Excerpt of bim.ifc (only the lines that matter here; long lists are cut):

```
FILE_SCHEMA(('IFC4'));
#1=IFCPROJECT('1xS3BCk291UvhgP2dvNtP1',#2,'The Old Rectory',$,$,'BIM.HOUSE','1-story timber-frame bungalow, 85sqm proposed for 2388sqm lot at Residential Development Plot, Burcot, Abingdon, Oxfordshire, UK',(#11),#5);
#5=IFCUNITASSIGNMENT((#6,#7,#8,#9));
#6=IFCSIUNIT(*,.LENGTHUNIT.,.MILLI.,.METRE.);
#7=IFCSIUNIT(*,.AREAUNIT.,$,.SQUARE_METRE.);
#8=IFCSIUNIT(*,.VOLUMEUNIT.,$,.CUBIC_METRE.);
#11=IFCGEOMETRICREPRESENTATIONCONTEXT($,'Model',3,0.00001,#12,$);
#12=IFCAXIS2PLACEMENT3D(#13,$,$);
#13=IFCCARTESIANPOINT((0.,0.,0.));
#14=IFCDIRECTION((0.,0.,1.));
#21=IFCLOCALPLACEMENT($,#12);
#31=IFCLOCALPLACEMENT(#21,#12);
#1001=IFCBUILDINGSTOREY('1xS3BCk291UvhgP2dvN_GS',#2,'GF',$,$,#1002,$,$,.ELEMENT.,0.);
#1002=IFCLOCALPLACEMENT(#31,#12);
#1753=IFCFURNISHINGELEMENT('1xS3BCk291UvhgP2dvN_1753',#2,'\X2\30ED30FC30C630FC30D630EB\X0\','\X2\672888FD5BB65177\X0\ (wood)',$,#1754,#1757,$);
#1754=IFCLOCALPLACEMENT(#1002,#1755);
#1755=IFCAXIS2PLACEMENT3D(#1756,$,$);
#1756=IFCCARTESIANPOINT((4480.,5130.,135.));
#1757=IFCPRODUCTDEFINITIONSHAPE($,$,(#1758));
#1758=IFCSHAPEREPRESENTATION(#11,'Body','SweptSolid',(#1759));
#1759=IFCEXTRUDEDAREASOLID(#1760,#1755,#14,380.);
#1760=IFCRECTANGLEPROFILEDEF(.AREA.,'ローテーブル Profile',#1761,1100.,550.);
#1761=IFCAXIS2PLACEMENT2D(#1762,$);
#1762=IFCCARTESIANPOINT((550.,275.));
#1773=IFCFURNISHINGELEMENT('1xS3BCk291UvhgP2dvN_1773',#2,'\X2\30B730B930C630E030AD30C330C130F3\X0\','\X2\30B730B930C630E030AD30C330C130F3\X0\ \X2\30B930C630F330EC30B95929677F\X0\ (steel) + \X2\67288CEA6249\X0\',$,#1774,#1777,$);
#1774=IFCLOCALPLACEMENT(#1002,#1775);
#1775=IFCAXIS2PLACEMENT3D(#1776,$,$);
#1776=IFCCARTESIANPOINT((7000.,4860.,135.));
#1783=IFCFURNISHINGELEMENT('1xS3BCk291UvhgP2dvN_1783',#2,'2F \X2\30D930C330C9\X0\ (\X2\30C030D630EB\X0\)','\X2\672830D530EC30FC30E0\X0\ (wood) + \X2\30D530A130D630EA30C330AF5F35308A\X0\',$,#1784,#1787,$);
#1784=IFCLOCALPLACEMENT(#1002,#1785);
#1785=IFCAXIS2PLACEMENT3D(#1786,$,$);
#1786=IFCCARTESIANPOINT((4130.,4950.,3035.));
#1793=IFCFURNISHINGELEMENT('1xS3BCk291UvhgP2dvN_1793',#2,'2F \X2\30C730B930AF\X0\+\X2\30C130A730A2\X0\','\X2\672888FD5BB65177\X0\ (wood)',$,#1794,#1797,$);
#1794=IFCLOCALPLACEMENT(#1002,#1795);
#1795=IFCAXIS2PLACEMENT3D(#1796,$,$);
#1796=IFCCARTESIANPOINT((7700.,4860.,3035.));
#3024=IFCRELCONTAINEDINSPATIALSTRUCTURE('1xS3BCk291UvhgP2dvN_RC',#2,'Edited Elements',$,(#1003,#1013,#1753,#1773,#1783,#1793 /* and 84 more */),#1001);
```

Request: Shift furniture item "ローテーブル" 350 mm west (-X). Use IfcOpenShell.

```python
import ifcopenshell
import ifcopenshell.api.geometry
import ifcopenshell.util.placement
import ifcopenshell.util.unit

model = ifcopenshell.open("bim.ifc")
unit_scale = ifcopenshell.util.unit.calculate_unit_scale(model)

item = model.by_guid("1xS3BCk291UvhgP2dvN_1753")
matrix = ifcopenshell.util.placement.get_local_placement(item.ObjectPlacement)
matrix[0, 3] -= 0.35 / unit_scale
ifcopenshell.api.geometry.edit_object_placement(model, product=item, matrix=matrix, is_si=False)

print(ifcopenshell.util.placement.get_local_placement(item.ObjectPlacement).round(3) + 0.0)

model.write("bim_edited.ifc")
```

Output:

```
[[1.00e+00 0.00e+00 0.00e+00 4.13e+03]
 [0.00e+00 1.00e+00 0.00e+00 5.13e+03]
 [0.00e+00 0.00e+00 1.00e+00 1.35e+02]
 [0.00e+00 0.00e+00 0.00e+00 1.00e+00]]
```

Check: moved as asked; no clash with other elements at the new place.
